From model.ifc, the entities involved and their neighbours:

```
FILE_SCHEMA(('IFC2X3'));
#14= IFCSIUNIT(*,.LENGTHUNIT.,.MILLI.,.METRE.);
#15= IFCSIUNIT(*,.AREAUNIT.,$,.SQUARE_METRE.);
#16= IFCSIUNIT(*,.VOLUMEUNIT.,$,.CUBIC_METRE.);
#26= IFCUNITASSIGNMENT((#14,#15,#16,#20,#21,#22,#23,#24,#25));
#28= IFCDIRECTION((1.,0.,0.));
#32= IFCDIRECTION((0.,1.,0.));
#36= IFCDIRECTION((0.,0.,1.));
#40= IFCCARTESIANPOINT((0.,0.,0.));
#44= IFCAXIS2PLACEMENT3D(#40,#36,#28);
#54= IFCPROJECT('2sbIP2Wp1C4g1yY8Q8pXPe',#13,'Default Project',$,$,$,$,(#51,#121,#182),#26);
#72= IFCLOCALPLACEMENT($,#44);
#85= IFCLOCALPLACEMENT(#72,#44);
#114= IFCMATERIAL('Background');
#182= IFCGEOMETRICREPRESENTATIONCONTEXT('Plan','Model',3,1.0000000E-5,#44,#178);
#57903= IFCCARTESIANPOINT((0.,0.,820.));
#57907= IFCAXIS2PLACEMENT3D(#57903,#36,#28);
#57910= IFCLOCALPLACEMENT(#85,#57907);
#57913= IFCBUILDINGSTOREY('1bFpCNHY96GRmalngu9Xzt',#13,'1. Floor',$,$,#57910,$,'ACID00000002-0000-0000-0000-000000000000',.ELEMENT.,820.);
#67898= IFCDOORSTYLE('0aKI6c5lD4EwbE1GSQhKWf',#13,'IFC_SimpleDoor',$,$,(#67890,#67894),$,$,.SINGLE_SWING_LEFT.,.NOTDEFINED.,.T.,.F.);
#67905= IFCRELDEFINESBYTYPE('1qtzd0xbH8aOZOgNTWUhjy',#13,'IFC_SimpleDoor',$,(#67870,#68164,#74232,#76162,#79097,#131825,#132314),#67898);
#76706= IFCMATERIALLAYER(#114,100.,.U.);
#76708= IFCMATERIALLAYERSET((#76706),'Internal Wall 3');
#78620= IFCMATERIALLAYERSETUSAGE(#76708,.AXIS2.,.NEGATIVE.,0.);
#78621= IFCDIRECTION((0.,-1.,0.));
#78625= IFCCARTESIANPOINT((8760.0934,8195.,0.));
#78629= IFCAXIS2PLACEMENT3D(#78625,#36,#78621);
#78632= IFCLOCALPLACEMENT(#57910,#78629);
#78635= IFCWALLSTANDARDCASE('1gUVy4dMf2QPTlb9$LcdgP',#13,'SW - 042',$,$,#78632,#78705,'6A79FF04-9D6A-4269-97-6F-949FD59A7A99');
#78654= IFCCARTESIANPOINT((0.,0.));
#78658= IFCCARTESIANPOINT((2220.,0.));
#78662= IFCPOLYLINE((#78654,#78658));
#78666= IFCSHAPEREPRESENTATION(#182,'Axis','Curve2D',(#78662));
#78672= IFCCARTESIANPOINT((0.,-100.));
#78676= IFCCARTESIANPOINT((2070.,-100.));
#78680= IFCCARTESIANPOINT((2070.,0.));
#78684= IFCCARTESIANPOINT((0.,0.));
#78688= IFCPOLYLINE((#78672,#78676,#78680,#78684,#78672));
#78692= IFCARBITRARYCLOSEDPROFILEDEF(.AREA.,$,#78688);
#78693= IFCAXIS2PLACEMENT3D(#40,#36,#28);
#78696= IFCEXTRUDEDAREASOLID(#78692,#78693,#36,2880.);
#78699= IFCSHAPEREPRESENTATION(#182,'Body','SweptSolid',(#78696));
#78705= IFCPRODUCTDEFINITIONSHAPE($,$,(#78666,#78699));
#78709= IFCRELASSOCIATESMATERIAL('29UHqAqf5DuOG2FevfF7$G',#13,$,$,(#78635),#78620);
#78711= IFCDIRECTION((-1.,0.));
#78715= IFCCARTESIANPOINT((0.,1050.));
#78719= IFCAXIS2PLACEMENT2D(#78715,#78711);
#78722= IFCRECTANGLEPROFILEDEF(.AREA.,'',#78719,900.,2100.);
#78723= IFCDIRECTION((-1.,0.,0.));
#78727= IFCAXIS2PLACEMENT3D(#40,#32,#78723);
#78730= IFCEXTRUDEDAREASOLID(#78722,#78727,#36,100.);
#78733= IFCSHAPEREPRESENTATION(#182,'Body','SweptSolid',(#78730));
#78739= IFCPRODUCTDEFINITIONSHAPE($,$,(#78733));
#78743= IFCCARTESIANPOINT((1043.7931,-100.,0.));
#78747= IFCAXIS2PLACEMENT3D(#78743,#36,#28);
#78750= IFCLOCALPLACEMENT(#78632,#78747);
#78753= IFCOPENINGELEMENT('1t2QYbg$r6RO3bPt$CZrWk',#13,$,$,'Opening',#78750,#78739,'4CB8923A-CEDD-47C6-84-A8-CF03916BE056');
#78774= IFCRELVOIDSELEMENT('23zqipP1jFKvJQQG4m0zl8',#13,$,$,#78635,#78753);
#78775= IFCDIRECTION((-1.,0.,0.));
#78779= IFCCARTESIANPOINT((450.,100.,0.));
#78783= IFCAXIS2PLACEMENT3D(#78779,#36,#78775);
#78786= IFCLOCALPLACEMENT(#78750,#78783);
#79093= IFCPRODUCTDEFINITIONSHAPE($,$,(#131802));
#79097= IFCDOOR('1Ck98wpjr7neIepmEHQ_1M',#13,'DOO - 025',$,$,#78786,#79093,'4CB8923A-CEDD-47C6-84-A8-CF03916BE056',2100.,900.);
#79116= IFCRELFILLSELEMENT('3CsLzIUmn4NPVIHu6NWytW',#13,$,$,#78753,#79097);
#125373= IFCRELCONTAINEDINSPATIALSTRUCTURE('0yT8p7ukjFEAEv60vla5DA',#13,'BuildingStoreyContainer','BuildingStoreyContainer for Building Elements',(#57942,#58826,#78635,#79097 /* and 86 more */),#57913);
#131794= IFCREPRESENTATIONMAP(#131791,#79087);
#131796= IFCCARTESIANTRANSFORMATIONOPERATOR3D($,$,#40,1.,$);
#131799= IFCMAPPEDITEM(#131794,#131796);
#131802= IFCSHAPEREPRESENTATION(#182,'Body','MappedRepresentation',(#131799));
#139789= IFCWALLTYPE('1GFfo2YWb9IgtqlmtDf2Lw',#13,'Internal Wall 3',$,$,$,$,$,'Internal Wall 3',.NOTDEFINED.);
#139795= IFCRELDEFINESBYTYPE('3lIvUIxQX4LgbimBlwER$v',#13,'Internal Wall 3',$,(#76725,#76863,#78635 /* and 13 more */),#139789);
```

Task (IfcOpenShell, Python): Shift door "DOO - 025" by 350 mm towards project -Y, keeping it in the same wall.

```python
import ifcopenshell
import ifcopenshell.api.geometry
import ifcopenshell.util.placement

model = ifcopenshell.open("model.ifc")

door = model.by_guid("1Ck98wpjr7neIepmEHQ_1M")
opening = door.FillsVoids[0].RelatingOpeningElement
wall = opening.VoidsElements[0].RelatingBuildingElement

wall_matrix = ifcopenshell.util.placement.get_local_placement(wall.ObjectPlacement)
shift = wall_matrix[:3, 0] * 350.0
before = ifcopenshell.util.placement.get_local_placement(door.ObjectPlacement)[:3, 3].copy()

# The door is placed relative to its opening, so it follows when the opening moves.
matrix = ifcopenshell.util.placement.get_local_placement(opening.ObjectPlacement)
matrix[:3, 3] += shift
ifcopenshell.api.geometry.edit_object_placement(
    model, product=opening, matrix=matrix, is_si=False, should_transform_children=True
)

after = ifcopenshell.util.placement.get_local_placement(door.ObjectPlacement)[:3, 3]
print("door moved by", (after - before).round(3) + 0.0)

model.write("model_v2.ifc")
```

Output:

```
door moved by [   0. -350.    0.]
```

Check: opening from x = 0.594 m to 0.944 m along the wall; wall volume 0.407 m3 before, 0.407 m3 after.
